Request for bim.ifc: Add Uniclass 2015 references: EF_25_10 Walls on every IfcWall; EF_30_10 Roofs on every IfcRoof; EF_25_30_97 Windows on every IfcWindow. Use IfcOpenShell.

First a look at what the model holds.

```python
import ifcopenshell

model = ifcopenshell.open("bim.ifc")
print(model.schema)
print("classifications:", [c.Name for c in model.by_type("IfcClassification")])
for ifc_class in ("IfcDoor", "IfcRoof", "IfcStair", "IfcWall", "IfcWindow"):
    print(ifc_class, len(model.by_type(ifc_class)))
```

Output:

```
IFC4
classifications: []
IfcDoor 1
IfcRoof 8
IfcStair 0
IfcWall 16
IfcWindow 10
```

```python
import ifcopenshell
import ifcopenshell.api.classification

model = ifcopenshell.open("bim.ifc")

system = ifcopenshell.api.classification.add_classification(model, classification="Uniclass 2015")

codes = {
    "IfcWall": ("EF_25_10", "Walls"),
    "IfcRoof": ("EF_30_10", "Roofs"),
    "IfcWindow": ("EF_25_30_97", "Windows"),
}
for ifc_class, (code, name) in codes.items():
    products = model.by_type(ifc_class)
    ifcopenshell.api.classification.add_reference(
        model, products=products, classification=system, identification=code, name=name
    )
    print(code, len(products))

model.write("bim-out.ifc")
```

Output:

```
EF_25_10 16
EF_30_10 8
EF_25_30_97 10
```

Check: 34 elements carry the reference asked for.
